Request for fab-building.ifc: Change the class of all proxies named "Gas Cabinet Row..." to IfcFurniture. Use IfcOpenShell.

First a look at what the model holds.

```python
import re

import ifcopenshell

model = ifcopenshell.open("fab-building.ifc")
print(model.schema)
seen = {}
for e in model.by_type("IfcBuildingElementProxy"):
    name = re.sub(r":\d+(:\d+)?$", "", e.Name or "")  # drop the element id that some exporters append
    seen[name] = seen.get(name, 0) + 1
for name, count in sorted(seen.items()):
    print(count, "x", name)
```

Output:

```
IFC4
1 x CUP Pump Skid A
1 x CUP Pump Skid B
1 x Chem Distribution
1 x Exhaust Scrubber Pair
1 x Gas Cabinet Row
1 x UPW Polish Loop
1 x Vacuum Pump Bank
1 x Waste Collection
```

```python
import ifcopenshell
import ifcopenshell.api.root

model = ifcopenshell.open("fab-building.ifc")

proxies = [e.id() for e in model.by_type("IfcBuildingElementProxy") if (e.Name or "").startswith("Gas Cabinet Row")]
for step_id in proxies:
    proxy = model.by_id(step_id)
    ifcopenshell.api.root.reassign_class(model, product=proxy, ifc_class="IfcFurniture")

print(sum(model.by_id(i).is_a("IfcFurniture") for i in proxies), "reclassified")

model.write("fab-building_edited.ifc")
```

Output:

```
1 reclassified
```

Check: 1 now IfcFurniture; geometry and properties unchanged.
